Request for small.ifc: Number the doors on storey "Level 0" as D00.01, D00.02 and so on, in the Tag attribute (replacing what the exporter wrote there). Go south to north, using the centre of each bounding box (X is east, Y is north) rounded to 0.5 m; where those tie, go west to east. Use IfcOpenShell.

First a look at what the model holds.

```python
import ifcopenshell
import ifcopenshell.util.element
import ifcopenshell.util.placement

model = ifcopenshell.open("small.ifc")
print(model.schema)
storey = next(s for s in model.by_type("IfcBuildingStorey") if s.Name == "Level 0")
doors = [e for e in ifcopenshell.util.element.get_decomposition(storey) if e.is_a("IfcDoor")]
for e in sorted(doors, key=lambda e: e.id()):
    origin = ifcopenshell.util.placement.get_local_placement(e.ObjectPlacement)[:3, 3]
    print(e.id(), e.Tag, e.Name, origin.round(2) + 0.0, sep=" | ")
```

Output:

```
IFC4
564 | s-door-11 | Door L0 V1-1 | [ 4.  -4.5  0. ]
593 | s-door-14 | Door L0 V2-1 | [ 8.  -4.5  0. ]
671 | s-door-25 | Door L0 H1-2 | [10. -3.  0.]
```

```python
import ifcopenshell
import ifcopenshell.geom
import ifcopenshell.util.element
import ifcopenshell.util.shape

model = ifcopenshell.open("small.ifc")
settings = ifcopenshell.geom.settings()
settings.set("use-world-coords", True)


def centre(element):
    shape = ifcopenshell.geom.create_shape(settings, element)
    return ifcopenshell.util.shape.get_bbox_centroid(shape.geometry)


storey = next(s for s in model.by_type("IfcBuildingStorey") if s.Name == "Level 0")
doors = [e for e in ifcopenshell.util.element.get_decomposition(storey) if e.is_a("IfcDoor")]

# Insertion points can sit at a corner or the storey origin, so sort by the geometry (in metres).
centres = {e: centre(e) for e in doors}
doors.sort(key=lambda e: (round(centres[e][1] / 0.5), centres[e][0]))

for i, e in enumerate(doors, start=1):
    number = f"D00.{i:02d}"
    e.Tag = number
    print(e.id(), number)

model.write("small-out.ifc")
```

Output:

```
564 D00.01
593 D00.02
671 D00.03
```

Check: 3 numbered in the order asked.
